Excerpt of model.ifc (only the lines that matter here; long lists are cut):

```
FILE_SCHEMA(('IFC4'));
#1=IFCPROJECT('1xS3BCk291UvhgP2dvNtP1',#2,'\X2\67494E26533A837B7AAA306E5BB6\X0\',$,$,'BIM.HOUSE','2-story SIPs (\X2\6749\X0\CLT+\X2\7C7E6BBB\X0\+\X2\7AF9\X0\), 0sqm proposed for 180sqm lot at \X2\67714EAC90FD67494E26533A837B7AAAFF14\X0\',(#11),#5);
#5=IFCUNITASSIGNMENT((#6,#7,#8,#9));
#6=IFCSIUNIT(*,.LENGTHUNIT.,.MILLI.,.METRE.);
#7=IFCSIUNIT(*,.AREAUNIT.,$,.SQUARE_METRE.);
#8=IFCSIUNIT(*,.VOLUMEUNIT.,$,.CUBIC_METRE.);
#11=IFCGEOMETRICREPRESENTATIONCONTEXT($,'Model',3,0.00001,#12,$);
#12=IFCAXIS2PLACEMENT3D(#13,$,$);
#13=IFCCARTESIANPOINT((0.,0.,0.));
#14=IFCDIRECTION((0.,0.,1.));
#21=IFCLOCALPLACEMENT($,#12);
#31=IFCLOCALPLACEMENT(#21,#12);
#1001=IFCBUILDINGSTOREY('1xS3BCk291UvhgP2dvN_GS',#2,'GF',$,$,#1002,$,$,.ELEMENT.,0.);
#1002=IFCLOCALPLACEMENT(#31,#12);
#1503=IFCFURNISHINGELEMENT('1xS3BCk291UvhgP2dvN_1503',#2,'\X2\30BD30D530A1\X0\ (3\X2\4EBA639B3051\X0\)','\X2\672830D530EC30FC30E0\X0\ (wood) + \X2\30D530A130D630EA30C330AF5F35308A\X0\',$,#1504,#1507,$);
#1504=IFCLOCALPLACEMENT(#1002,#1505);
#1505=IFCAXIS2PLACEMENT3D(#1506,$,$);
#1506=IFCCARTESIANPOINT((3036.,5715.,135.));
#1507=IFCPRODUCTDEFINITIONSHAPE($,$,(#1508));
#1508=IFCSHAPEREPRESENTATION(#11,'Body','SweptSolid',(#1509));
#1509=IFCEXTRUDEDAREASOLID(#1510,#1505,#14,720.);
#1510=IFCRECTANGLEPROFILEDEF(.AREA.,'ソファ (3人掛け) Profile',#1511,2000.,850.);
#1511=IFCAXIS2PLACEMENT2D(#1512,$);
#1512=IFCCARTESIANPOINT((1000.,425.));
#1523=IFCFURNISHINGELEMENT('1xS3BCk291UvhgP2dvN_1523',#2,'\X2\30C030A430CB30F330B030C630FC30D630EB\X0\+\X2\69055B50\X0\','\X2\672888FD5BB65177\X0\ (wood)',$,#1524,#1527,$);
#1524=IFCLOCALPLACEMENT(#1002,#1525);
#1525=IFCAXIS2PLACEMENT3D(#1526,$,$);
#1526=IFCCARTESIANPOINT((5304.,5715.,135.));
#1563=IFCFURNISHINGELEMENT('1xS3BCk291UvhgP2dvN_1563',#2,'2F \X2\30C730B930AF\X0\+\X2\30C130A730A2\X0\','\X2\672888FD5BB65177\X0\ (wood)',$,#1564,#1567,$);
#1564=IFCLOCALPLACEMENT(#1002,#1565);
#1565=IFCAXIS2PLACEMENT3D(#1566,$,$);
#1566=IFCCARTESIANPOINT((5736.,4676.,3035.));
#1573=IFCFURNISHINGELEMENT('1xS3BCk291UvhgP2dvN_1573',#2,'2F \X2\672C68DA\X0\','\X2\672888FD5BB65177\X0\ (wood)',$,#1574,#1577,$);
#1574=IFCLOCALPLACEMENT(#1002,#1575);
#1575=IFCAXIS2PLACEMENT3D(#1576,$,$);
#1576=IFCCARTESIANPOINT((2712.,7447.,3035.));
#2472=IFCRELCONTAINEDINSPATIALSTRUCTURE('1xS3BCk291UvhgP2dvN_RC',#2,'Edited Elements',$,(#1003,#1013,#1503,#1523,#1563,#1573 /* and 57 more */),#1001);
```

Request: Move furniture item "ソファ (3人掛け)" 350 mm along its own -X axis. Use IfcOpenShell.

```python
import ifcopenshell
import ifcopenshell.api.geometry
import ifcopenshell.util.placement
import ifcopenshell.util.unit

model = ifcopenshell.open("model.ifc")
unit_scale = ifcopenshell.util.unit.calculate_unit_scale(model)

item = model.by_guid("1xS3BCk291UvhgP2dvN_1503")
matrix = ifcopenshell.util.placement.get_local_placement(item.ObjectPlacement)
matrix[:3, 3] -= matrix[:3, 0] * 0.35 / unit_scale
ifcopenshell.api.geometry.edit_object_placement(model, product=item, matrix=matrix, is_si=False)

print(ifcopenshell.util.placement.get_local_placement(item.ObjectPlacement).round(3) + 0.0)

model.write("model_rev.ifc")
```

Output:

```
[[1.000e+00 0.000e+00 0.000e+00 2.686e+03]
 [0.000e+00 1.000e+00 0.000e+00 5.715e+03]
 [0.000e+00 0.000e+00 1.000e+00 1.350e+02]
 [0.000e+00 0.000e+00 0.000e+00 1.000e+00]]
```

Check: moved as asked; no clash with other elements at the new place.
